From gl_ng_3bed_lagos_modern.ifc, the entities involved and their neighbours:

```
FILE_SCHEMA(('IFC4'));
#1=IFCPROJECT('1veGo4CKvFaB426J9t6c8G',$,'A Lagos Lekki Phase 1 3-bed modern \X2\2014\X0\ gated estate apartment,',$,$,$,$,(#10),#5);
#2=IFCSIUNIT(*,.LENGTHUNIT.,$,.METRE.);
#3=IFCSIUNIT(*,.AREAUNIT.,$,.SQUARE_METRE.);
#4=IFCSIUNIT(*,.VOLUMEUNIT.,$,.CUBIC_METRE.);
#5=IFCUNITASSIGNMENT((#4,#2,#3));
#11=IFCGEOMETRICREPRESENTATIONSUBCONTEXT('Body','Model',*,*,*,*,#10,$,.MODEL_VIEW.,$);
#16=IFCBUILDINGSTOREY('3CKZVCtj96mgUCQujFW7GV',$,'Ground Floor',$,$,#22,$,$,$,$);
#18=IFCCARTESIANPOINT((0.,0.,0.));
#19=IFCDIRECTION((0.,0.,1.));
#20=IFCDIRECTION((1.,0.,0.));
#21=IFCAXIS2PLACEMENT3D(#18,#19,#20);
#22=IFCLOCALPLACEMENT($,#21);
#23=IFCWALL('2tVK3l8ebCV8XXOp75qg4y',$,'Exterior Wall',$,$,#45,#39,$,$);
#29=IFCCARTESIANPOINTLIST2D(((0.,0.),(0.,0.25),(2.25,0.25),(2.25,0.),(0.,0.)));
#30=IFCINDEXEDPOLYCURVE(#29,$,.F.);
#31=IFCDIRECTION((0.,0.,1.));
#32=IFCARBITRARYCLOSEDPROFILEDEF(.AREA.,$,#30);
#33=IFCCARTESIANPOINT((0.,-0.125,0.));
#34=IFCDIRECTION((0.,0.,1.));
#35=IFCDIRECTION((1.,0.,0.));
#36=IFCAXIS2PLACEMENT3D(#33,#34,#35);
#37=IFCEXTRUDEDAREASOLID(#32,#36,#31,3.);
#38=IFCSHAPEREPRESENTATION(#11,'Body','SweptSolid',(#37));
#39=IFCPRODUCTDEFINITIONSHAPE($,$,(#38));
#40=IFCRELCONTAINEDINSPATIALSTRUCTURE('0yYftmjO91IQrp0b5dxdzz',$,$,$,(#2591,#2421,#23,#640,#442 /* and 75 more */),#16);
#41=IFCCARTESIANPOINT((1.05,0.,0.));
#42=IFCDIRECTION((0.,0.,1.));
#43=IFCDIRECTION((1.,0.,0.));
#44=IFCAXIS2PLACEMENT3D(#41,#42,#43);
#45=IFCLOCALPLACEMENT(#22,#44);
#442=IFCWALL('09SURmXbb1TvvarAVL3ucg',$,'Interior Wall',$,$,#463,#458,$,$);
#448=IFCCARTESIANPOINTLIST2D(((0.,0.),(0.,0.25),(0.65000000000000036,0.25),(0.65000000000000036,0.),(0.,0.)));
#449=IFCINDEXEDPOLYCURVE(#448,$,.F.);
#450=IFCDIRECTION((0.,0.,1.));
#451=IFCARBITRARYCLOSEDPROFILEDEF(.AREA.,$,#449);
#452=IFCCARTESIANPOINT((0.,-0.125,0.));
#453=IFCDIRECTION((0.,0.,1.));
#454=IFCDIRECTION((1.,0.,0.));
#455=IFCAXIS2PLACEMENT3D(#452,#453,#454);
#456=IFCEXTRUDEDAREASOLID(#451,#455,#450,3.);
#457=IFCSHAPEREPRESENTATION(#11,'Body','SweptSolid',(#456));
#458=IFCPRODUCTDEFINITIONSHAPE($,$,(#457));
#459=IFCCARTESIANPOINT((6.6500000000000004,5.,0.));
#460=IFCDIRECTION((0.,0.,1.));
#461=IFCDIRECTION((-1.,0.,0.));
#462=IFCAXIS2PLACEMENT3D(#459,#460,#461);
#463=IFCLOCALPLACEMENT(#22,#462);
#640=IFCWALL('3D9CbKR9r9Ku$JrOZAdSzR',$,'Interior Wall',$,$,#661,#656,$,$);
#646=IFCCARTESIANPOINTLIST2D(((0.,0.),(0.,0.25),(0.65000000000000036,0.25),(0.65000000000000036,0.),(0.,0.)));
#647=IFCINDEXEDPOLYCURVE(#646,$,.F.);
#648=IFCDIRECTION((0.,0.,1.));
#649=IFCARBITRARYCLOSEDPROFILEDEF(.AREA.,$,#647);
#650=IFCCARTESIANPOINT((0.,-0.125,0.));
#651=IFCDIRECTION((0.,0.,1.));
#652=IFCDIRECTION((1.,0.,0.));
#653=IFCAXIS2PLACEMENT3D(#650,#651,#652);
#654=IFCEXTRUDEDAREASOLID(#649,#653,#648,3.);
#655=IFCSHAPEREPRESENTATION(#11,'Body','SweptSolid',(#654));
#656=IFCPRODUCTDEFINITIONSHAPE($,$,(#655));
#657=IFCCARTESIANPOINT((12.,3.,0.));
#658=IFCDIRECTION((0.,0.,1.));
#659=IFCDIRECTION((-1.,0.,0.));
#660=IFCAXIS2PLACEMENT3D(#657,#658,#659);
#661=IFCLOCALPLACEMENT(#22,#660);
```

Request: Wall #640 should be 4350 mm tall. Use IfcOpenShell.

```python
import ifcopenshell
import ifcopenshell.geom
import ifcopenshell.util.representation
import ifcopenshell.util.shape
import ifcopenshell.util.unit

model = ifcopenshell.open("gl_ng_3bed_lagos_modern.ifc")
unit_scale = ifcopenshell.util.unit.calculate_unit_scale(model)
settings = ifcopenshell.geom.settings()


def volume(element):
    """Net volume in cubic metres, openings subtracted."""
    shape = ifcopenshell.geom.create_shape(settings, element)
    return ifcopenshell.util.shape.get_volume(shape.geometry)


wall = model.by_guid("3D9CbKR9r9Ku$JrOZAdSzR")
before = volume(wall)

body = ifcopenshell.util.representation.get_representation(wall, "Model", "Body")
solid = body.Items[0]
old_height = solid.Depth
solid.Depth = 4.35 / unit_scale
after = volume(wall)

print(f"height {old_height:g} -> {solid.Depth:g}, volume {before:.3f} -> {after:.3f} m3")

model.write("gl_ng_3bed_lagos_modern_v2.ifc")
```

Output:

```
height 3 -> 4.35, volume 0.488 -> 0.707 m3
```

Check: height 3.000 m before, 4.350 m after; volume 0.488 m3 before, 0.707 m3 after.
